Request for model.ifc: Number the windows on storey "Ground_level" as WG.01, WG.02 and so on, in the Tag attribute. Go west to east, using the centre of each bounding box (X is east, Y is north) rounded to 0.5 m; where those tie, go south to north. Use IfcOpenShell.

First a look at what the model holds.

```python
import ifcopenshell
import ifcopenshell.util.element
import ifcopenshell.util.placement

model = ifcopenshell.open("model.ifc")
print(model.schema)
storey = next(s for s in model.by_type("IfcBuildingStorey") if s.Name == "Ground_level")
windows = [e for e in ifcopenshell.util.element.get_decomposition(storey) if e.is_a("IfcWindow")]
for e in sorted(windows, key=lambda e: e.id()):
    origin = ifcopenshell.util.placement.get_local_placement(e.ObjectPlacement)[:3, 3]
    print(e.id(), e.Tag, e.Name, origin.round(2) + 0.0, sep=" | ")
```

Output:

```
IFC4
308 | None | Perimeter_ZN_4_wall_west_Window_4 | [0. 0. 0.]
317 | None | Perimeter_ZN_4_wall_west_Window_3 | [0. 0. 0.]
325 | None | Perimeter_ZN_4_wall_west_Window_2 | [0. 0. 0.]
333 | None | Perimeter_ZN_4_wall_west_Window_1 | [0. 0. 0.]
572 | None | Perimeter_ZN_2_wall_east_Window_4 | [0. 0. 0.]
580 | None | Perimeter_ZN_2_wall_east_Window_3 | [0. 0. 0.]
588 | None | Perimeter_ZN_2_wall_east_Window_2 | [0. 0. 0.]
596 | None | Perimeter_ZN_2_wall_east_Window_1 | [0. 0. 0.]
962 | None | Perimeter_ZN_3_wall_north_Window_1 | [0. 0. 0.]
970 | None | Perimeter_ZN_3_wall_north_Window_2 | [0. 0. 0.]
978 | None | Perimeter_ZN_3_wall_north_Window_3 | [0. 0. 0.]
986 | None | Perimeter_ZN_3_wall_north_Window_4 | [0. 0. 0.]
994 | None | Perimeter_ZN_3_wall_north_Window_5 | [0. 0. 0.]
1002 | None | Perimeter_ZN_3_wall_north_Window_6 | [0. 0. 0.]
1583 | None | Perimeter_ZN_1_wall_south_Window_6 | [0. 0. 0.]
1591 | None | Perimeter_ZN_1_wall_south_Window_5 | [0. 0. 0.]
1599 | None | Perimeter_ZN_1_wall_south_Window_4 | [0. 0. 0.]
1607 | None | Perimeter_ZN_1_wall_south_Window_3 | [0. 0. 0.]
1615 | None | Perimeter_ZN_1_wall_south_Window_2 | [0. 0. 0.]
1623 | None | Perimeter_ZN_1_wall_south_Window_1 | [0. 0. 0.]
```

```python
import ifcopenshell
import ifcopenshell.geom
import ifcopenshell.util.element
import ifcopenshell.util.shape

model = ifcopenshell.open("model.ifc")
settings = ifcopenshell.geom.settings()
settings.set("use-world-coords", True)


def centre(element):
    shape = ifcopenshell.geom.create_shape(settings, element)
    return ifcopenshell.util.shape.get_bbox_centroid(shape.geometry)


storey = next(s for s in model.by_type("IfcBuildingStorey") if s.Name == "Ground_level")
windows = [e for e in ifcopenshell.util.element.get_decomposition(storey) if e.is_a("IfcWindow")]

# Insertion points can sit at a corner or the storey origin, so sort by the geometry (in metres).
centres = {e: centre(e) for e in windows}
windows.sort(key=lambda e: (round(centres[e][0] / 0.5), centres[e][1]))

for i, e in enumerate(windows, start=1):
    number = f"WG.{i:02d}"
    e.Tag = number
    print(e.id(), number)

model.write("model_edited.ifc")
```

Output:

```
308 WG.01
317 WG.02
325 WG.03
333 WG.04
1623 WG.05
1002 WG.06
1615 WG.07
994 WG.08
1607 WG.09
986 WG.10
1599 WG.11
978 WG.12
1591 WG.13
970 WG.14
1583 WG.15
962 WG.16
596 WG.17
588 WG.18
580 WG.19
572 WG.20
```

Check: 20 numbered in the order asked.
